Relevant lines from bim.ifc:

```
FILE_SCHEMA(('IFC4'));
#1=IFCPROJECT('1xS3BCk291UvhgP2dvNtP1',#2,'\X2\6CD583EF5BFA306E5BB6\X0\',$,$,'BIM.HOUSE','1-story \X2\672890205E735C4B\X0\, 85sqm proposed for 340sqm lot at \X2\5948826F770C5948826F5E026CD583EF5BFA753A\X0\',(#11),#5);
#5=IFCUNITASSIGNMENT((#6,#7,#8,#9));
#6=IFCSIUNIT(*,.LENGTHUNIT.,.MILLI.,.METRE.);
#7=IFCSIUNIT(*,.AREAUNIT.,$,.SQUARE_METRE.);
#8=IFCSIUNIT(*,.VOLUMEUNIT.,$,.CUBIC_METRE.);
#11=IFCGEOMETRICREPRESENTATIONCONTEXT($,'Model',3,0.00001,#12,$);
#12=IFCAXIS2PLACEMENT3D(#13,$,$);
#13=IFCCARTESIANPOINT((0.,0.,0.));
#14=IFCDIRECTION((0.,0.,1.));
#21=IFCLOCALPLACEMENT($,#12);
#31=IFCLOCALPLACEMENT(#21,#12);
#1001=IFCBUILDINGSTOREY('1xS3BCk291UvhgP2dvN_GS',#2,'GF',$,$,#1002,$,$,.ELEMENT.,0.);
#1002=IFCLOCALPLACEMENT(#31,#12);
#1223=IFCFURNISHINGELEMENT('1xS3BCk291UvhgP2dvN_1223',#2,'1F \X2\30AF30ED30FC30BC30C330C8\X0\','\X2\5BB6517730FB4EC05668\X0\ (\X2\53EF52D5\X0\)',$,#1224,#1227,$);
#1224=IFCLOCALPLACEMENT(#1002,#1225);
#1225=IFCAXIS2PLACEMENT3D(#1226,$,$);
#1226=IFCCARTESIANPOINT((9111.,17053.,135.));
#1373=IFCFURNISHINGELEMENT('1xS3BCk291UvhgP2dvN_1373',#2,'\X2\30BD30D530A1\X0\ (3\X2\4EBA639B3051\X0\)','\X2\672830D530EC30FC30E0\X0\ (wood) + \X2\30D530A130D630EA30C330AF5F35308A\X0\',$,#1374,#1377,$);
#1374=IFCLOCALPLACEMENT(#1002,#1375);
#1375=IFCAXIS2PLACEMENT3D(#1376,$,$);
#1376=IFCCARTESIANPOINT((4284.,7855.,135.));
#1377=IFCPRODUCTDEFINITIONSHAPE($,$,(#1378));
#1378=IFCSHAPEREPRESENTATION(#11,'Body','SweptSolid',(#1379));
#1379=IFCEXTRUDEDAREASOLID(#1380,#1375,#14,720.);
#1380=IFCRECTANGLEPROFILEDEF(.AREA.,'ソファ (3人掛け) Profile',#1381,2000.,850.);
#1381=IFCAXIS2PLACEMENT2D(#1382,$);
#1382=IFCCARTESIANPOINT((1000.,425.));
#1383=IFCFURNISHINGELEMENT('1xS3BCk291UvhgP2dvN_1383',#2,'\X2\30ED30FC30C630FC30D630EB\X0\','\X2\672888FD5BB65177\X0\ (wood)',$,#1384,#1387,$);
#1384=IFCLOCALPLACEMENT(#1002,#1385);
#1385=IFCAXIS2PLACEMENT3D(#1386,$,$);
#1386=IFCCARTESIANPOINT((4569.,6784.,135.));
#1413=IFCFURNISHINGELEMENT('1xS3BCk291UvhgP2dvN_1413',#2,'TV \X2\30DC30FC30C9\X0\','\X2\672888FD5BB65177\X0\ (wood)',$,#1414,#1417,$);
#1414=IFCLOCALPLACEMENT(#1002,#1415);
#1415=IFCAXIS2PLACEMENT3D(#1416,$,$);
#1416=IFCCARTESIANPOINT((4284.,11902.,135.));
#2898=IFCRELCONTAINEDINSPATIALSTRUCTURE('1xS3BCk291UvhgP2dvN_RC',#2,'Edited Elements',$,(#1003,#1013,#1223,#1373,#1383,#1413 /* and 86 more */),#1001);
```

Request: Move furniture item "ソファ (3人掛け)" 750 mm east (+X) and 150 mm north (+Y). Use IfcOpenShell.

```python
import ifcopenshell
import ifcopenshell.api.geometry
import ifcopenshell.util.placement

model = ifcopenshell.open("bim.ifc")

item = model.by_guid("1xS3BCk291UvhgP2dvN_1373")
matrix = ifcopenshell.util.placement.get_local_placement(item.ObjectPlacement)
matrix[0, 3] += 750.0
matrix[1, 3] += 150.0
ifcopenshell.api.geometry.edit_object_placement(model, product=item, matrix=matrix, is_si=False)

print(ifcopenshell.util.placement.get_local_placement(item.ObjectPlacement).round(3) + 0.0)

model.write("bim_rev.ifc")
```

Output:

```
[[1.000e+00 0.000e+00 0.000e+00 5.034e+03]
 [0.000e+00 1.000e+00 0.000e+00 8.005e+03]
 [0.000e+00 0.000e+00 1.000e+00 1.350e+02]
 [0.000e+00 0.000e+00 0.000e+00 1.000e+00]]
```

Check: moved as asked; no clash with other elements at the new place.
